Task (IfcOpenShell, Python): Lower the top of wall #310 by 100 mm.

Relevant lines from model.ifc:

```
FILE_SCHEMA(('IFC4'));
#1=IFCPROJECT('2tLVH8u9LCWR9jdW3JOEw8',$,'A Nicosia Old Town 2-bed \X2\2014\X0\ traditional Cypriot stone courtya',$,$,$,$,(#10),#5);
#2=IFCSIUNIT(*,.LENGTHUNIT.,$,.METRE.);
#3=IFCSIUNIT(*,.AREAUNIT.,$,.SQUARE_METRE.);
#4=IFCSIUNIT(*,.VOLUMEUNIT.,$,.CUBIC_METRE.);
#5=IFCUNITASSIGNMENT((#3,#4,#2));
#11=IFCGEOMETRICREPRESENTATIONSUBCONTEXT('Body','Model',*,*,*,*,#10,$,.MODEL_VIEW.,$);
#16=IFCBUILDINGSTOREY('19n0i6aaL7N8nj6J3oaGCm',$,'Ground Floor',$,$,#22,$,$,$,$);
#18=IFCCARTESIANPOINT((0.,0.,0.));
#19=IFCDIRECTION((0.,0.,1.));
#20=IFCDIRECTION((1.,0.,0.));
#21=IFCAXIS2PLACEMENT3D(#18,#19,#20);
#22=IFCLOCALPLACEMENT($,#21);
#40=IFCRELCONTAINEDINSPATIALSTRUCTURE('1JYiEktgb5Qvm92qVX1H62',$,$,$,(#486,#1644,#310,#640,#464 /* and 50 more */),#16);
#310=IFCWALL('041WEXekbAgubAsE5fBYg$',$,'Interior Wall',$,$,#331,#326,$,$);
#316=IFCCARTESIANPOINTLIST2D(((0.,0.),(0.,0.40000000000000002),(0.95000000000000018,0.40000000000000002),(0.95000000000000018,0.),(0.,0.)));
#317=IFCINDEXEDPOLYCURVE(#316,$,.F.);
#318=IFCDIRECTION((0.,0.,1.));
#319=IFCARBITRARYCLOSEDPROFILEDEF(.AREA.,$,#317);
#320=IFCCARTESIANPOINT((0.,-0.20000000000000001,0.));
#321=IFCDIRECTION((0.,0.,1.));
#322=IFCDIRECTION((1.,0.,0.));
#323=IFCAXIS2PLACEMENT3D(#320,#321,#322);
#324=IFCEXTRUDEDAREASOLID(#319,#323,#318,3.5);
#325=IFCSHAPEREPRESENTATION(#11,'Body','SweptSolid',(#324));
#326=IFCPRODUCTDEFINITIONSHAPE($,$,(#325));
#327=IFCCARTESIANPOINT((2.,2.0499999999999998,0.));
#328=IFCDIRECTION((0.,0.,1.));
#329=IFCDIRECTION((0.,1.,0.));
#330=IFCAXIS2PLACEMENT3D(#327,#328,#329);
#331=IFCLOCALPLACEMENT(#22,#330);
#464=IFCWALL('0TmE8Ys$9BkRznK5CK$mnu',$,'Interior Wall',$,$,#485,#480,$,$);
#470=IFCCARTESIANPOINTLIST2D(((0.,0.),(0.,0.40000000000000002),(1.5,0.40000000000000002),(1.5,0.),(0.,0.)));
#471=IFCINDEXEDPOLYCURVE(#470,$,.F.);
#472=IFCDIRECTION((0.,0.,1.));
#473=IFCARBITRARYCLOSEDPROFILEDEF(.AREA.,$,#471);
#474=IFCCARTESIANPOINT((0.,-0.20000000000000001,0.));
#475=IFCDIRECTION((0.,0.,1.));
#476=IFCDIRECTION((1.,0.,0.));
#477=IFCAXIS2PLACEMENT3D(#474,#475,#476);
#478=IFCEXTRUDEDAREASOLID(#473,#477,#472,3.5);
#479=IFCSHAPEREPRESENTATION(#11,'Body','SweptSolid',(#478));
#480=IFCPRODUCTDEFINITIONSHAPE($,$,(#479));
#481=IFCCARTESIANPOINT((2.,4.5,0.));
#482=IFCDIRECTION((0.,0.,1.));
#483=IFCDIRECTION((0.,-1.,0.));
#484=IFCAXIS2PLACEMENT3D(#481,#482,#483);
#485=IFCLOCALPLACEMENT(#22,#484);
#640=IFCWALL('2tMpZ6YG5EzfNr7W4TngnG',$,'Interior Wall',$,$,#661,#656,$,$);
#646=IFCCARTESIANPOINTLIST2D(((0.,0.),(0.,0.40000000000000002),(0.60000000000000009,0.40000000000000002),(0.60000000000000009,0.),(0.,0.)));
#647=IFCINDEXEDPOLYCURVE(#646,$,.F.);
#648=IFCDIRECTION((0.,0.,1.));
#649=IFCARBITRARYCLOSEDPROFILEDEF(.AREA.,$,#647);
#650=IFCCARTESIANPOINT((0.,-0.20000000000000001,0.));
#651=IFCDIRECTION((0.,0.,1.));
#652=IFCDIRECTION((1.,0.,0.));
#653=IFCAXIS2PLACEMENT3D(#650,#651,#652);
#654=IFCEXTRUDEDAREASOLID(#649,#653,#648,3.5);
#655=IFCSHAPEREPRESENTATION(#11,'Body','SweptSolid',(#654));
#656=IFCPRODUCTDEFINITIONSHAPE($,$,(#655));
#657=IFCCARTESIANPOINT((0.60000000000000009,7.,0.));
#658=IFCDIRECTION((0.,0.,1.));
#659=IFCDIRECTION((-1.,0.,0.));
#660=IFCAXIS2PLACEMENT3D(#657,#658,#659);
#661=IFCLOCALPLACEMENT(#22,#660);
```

```python
import ifcopenshell
import ifcopenshell.geom
import ifcopenshell.util.representation
import ifcopenshell.util.shape
import ifcopenshell.util.unit

model = ifcopenshell.open("model.ifc")
unit_scale = ifcopenshell.util.unit.calculate_unit_scale(model)
settings = ifcopenshell.geom.settings()


def volume(element):
    """Net volume in cubic metres, openings subtracted."""
    shape = ifcopenshell.geom.create_shape(settings, element)
    return ifcopenshell.util.shape.get_volume(shape.geometry)


wall = model.by_id(310)
before = volume(wall)

body = ifcopenshell.util.representation.get_representation(wall, "Model", "Body")
solid = body.Items[0]
old_height = solid.Depth
solid.Depth -= 0.1 / unit_scale
after = volume(wall)

print(f"height {old_height:g} -> {solid.Depth:g}, volume {before:.3f} -> {after:.3f} m3")

model.write("model_v2.ifc")
```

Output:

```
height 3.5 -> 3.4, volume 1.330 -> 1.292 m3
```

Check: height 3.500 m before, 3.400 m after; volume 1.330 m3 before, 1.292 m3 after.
